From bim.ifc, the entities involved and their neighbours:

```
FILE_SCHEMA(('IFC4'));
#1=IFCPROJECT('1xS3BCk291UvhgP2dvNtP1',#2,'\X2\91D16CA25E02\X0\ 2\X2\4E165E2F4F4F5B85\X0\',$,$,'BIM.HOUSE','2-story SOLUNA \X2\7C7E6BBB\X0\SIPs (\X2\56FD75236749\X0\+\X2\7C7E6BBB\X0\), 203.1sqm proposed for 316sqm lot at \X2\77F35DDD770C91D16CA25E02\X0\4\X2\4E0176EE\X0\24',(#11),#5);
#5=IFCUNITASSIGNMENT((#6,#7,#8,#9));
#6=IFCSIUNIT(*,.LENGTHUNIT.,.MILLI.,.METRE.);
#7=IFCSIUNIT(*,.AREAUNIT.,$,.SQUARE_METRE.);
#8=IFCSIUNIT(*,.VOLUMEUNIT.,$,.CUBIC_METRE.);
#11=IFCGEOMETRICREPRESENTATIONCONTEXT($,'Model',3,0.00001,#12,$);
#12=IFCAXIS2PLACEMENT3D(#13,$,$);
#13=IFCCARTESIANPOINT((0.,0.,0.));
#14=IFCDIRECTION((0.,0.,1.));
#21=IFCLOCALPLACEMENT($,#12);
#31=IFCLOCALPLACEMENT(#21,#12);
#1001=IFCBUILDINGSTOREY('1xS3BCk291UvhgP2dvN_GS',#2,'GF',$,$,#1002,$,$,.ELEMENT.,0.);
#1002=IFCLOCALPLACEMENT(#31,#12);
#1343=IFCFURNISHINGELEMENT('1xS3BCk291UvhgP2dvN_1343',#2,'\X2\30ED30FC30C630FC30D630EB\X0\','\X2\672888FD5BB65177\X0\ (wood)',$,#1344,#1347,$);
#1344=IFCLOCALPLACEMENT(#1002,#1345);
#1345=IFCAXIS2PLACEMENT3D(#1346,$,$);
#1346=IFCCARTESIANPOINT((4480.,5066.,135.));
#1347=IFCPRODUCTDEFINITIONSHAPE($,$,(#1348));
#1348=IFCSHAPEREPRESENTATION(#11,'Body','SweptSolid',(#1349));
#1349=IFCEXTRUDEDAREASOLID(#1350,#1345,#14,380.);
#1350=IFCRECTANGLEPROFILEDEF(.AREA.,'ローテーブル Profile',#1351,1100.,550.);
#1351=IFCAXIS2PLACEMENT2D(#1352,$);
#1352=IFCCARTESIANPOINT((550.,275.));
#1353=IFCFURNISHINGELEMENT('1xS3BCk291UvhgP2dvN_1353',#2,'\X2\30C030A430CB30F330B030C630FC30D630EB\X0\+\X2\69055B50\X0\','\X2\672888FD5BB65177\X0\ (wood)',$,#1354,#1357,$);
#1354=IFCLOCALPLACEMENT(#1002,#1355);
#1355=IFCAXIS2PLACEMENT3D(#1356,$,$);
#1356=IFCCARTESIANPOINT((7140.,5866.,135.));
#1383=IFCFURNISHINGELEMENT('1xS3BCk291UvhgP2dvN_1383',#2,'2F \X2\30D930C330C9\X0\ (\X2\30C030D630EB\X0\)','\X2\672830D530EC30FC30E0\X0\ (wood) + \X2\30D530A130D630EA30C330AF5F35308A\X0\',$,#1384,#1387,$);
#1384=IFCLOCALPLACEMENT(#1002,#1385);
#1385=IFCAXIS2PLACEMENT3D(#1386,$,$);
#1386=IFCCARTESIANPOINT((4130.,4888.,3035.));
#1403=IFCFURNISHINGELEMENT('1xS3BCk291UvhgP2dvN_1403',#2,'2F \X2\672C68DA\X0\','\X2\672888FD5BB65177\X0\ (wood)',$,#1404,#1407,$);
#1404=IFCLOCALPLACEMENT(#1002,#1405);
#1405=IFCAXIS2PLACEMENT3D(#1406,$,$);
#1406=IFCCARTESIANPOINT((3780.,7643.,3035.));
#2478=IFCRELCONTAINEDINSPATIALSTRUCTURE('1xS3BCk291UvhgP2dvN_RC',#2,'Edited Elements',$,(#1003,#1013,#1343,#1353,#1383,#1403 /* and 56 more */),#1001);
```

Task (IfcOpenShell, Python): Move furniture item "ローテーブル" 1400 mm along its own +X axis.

```python
import ifcopenshell
import ifcopenshell.api.geometry
import ifcopenshell.util.placement

model = ifcopenshell.open("bim.ifc")

item = model.by_guid("1xS3BCk291UvhgP2dvN_1343")
matrix = ifcopenshell.util.placement.get_local_placement(item.ObjectPlacement)
matrix[:3, 3] += matrix[:3, 0] * 1400.0
ifcopenshell.api.geometry.edit_object_placement(model, product=item, matrix=matrix, is_si=False)

print(ifcopenshell.util.placement.get_local_placement(item.ObjectPlacement).round(3) + 0.0)

model.write("bim_v2.ifc")
```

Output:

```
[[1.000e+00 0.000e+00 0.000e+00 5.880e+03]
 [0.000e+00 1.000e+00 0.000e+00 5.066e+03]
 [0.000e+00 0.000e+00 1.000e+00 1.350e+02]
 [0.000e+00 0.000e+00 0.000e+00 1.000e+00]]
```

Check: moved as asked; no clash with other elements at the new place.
